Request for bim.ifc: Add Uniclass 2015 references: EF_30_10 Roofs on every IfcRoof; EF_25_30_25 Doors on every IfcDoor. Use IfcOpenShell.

First a look at what the model holds.

```python
import ifcopenshell

model = ifcopenshell.open("bim.ifc")
print(model.schema)
print("classifications:", [c.Name for c in model.by_type("IfcClassification")])
for ifc_class in ("IfcDoor", "IfcRoof", "IfcStair", "IfcWall", "IfcWindow"):
    print(ifc_class, len(model.by_type(ifc_class)))
```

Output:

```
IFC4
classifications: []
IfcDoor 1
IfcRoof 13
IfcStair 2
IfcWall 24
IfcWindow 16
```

```python
import ifcopenshell
import ifcopenshell.api.classification

model = ifcopenshell.open("bim.ifc")

system = ifcopenshell.api.classification.add_classification(model, classification="Uniclass 2015")

codes = {
    "IfcRoof": ("EF_30_10", "Roofs"),
    "IfcDoor": ("EF_25_30_25", "Doors"),
}
for ifc_class, (code, name) in codes.items():
    products = model.by_type(ifc_class)
    ifcopenshell.api.classification.add_reference(
        model, products=products, classification=system, identification=code, name=name
    )
    print(code, len(products))

model.write("bim_edited.ifc")
```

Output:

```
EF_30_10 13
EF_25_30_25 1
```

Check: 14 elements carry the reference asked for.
